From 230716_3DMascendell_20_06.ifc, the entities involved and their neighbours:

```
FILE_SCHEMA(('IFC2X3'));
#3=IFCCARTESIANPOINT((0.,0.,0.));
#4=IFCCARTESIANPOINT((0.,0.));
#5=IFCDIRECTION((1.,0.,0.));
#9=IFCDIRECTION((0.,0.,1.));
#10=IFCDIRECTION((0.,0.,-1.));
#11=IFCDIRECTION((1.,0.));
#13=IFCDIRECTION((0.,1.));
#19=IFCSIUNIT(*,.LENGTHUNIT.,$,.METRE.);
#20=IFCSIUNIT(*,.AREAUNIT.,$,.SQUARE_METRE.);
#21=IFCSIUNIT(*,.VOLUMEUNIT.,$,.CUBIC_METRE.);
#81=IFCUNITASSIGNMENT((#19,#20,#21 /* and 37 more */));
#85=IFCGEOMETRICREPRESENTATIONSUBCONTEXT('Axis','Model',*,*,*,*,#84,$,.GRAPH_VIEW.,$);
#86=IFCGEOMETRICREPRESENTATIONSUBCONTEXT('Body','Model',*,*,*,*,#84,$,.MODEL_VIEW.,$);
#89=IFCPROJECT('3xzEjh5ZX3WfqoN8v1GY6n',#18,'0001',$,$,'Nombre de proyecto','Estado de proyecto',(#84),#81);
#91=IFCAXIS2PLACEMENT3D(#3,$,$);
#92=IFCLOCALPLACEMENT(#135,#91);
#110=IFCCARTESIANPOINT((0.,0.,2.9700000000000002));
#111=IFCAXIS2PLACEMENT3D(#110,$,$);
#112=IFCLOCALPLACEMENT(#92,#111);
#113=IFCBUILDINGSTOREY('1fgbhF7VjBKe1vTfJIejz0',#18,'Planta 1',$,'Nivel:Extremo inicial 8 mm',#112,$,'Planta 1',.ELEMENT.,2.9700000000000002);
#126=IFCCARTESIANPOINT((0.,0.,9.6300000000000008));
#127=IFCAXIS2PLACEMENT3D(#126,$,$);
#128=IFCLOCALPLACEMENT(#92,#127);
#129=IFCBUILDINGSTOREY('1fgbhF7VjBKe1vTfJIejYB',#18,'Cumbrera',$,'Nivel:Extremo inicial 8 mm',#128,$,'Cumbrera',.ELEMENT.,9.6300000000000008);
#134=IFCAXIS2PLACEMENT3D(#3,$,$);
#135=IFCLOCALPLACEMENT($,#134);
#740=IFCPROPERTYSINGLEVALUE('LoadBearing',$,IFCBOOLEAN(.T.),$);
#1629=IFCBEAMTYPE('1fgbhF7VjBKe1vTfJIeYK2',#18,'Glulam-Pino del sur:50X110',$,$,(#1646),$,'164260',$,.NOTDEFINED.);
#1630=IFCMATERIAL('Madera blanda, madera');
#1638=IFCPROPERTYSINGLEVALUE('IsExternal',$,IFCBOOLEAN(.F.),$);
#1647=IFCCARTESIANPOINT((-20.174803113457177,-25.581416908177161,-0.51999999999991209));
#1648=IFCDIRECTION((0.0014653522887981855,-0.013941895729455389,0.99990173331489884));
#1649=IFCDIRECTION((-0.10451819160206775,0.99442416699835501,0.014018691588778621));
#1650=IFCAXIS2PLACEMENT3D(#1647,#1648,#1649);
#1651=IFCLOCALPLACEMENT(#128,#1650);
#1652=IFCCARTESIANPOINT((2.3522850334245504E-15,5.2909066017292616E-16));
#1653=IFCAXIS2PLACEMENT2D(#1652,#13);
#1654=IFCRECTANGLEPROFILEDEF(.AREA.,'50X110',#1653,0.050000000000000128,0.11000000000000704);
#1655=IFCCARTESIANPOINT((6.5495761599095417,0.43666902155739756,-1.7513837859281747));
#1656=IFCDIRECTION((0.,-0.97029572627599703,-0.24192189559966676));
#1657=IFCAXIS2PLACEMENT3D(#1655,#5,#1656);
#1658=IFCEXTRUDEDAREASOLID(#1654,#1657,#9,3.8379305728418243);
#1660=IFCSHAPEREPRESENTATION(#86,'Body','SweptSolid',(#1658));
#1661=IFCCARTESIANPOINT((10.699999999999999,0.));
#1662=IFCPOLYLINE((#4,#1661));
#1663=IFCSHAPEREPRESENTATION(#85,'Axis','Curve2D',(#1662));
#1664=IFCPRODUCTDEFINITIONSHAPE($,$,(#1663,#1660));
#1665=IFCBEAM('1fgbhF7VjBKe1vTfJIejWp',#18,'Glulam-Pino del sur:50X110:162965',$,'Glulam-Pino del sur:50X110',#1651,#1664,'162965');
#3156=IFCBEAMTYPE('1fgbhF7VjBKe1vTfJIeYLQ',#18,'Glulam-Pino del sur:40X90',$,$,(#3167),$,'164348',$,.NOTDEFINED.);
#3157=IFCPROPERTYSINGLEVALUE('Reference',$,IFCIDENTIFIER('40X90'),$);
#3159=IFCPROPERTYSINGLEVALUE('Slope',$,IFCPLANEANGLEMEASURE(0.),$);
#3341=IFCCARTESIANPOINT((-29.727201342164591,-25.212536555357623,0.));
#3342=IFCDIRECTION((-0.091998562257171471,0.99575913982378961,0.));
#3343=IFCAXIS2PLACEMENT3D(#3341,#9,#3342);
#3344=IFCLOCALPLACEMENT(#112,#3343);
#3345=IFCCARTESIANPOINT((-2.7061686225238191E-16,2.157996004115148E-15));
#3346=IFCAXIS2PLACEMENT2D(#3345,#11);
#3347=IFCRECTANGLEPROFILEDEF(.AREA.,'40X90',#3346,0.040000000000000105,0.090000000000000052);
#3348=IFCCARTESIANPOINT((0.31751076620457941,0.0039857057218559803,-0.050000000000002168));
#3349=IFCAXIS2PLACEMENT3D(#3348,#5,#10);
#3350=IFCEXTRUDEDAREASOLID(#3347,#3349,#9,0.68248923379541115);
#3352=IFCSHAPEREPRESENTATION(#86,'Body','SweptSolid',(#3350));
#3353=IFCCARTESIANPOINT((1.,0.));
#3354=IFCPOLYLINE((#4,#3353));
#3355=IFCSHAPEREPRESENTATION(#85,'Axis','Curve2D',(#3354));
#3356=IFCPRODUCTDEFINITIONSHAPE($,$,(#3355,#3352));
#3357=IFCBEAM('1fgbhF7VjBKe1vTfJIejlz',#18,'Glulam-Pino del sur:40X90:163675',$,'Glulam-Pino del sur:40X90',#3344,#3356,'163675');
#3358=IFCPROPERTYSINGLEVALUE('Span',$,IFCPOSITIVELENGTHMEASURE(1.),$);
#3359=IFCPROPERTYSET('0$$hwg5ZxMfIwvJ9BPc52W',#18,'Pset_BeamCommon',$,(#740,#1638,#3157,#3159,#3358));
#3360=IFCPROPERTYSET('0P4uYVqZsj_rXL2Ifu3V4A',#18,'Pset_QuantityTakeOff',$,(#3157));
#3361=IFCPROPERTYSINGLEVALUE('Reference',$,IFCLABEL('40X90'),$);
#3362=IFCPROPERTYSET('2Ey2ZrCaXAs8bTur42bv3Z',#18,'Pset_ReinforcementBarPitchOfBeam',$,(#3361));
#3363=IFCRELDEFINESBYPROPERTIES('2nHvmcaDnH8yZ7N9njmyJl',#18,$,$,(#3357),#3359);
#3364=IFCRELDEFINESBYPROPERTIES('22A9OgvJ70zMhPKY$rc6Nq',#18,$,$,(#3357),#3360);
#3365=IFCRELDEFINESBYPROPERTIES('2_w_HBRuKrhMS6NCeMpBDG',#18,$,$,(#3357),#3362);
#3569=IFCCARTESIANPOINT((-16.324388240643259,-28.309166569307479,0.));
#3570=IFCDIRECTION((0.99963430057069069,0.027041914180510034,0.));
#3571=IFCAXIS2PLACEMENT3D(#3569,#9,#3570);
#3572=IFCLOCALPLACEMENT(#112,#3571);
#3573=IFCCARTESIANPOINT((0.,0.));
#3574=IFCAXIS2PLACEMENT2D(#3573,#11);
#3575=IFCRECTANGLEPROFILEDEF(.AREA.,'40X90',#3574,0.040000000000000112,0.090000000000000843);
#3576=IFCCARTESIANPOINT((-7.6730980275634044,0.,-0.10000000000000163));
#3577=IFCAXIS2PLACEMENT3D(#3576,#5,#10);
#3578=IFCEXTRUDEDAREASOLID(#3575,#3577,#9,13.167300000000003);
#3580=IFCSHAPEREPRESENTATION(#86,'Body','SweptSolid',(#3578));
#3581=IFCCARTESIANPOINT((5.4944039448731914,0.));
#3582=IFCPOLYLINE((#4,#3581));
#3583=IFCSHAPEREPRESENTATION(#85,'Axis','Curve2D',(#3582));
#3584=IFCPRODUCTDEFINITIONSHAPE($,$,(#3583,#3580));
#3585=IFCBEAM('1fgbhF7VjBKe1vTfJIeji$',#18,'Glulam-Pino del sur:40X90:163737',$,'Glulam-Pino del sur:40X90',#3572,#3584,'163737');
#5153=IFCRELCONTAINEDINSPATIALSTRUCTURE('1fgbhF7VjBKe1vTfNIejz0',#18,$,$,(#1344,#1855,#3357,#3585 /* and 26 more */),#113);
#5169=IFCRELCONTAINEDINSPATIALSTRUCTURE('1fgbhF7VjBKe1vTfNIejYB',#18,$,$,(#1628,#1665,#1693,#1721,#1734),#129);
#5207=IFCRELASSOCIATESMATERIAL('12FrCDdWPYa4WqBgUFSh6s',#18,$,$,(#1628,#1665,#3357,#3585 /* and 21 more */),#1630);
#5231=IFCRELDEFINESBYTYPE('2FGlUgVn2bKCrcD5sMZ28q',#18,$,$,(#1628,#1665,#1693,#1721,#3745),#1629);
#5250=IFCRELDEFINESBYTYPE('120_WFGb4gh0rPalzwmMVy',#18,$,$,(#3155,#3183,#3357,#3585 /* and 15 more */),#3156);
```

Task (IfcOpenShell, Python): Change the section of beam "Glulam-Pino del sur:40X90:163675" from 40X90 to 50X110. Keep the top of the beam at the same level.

```python
import ifcopenshell
import ifcopenshell.api.pset
import ifcopenshell.api.type
import ifcopenshell.util.element
import ifcopenshell.util.representation

model = ifcopenshell.open("230716_3DMascendell_20_06.ifc")

member = model.by_guid("1fgbhF7VjBKe1vTfJIejlz")
source = next(p for p in model.by_type("IfcRectangleProfileDef") if p.ProfileName == "50X110")

body = ifcopenshell.util.representation.get_representation(member, "Model", "Body")
solid = body.Items[0]
old_profile = solid.SweptArea

# Copy the section's sizes but keep this member's own profile position.
profile = ifcopenshell.util.element.copy(model, source)
# Profiles are centred, so shift by half the change in depth to hold the top.
shift = (old_profile.XDim - profile.XDim) / 2
x, y = old_profile.Position.Location.Coordinates
up = (-1.0, 0.0)  # upwards, in the solid's own plane
location = model.createIfcCartesianPoint((x + up[0] * shift, y + up[1] * shift))
profile.Position = model.createIfcAxis2Placement2D(location, old_profile.Position.RefDirection)
solid.SweptArea = profile
if not model.get_total_inverses(old_profile):
    ifcopenshell.util.element.remove_deep2(model, old_profile)

new_type = model.by_guid("1fgbhF7VjBKe1vTfJIeYK2")
ifcopenshell.api.type.assign_type(
    model, related_objects=[member], relating_type=new_type, should_map_representations=False
)
member.Name = member.Name.replace("40X90", "50X110")
member.ObjectType = "Glulam-Pino del sur:50X110"
pset = model.by_id(ifcopenshell.util.element.get_pset(member, "Pset_BeamCommon", should_inherit=False)["id"])
ifcopenshell.api.pset.edit_pset(model, pset=pset, properties={"Reference": "50X110"})
pset = model.by_id(ifcopenshell.util.element.get_pset(member, "Pset_QuantityTakeOff", should_inherit=False)["id"])
ifcopenshell.api.pset.edit_pset(model, pset=pset, properties={"Reference": "50X110"})
pset = model.by_id(ifcopenshell.util.element.get_pset(member, "Pset_ReinforcementBarPitchOfBeam", should_inherit=False)["id"])
ifcopenshell.api.pset.edit_pset(model, pset=pset, properties={"Reference": "50X110"})

print(solid.SweptArea)

model.write("230716_3DMascendell_20_06_v2.ifc")
```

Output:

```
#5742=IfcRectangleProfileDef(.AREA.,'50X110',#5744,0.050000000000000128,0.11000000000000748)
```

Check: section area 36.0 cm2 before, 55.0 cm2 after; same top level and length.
